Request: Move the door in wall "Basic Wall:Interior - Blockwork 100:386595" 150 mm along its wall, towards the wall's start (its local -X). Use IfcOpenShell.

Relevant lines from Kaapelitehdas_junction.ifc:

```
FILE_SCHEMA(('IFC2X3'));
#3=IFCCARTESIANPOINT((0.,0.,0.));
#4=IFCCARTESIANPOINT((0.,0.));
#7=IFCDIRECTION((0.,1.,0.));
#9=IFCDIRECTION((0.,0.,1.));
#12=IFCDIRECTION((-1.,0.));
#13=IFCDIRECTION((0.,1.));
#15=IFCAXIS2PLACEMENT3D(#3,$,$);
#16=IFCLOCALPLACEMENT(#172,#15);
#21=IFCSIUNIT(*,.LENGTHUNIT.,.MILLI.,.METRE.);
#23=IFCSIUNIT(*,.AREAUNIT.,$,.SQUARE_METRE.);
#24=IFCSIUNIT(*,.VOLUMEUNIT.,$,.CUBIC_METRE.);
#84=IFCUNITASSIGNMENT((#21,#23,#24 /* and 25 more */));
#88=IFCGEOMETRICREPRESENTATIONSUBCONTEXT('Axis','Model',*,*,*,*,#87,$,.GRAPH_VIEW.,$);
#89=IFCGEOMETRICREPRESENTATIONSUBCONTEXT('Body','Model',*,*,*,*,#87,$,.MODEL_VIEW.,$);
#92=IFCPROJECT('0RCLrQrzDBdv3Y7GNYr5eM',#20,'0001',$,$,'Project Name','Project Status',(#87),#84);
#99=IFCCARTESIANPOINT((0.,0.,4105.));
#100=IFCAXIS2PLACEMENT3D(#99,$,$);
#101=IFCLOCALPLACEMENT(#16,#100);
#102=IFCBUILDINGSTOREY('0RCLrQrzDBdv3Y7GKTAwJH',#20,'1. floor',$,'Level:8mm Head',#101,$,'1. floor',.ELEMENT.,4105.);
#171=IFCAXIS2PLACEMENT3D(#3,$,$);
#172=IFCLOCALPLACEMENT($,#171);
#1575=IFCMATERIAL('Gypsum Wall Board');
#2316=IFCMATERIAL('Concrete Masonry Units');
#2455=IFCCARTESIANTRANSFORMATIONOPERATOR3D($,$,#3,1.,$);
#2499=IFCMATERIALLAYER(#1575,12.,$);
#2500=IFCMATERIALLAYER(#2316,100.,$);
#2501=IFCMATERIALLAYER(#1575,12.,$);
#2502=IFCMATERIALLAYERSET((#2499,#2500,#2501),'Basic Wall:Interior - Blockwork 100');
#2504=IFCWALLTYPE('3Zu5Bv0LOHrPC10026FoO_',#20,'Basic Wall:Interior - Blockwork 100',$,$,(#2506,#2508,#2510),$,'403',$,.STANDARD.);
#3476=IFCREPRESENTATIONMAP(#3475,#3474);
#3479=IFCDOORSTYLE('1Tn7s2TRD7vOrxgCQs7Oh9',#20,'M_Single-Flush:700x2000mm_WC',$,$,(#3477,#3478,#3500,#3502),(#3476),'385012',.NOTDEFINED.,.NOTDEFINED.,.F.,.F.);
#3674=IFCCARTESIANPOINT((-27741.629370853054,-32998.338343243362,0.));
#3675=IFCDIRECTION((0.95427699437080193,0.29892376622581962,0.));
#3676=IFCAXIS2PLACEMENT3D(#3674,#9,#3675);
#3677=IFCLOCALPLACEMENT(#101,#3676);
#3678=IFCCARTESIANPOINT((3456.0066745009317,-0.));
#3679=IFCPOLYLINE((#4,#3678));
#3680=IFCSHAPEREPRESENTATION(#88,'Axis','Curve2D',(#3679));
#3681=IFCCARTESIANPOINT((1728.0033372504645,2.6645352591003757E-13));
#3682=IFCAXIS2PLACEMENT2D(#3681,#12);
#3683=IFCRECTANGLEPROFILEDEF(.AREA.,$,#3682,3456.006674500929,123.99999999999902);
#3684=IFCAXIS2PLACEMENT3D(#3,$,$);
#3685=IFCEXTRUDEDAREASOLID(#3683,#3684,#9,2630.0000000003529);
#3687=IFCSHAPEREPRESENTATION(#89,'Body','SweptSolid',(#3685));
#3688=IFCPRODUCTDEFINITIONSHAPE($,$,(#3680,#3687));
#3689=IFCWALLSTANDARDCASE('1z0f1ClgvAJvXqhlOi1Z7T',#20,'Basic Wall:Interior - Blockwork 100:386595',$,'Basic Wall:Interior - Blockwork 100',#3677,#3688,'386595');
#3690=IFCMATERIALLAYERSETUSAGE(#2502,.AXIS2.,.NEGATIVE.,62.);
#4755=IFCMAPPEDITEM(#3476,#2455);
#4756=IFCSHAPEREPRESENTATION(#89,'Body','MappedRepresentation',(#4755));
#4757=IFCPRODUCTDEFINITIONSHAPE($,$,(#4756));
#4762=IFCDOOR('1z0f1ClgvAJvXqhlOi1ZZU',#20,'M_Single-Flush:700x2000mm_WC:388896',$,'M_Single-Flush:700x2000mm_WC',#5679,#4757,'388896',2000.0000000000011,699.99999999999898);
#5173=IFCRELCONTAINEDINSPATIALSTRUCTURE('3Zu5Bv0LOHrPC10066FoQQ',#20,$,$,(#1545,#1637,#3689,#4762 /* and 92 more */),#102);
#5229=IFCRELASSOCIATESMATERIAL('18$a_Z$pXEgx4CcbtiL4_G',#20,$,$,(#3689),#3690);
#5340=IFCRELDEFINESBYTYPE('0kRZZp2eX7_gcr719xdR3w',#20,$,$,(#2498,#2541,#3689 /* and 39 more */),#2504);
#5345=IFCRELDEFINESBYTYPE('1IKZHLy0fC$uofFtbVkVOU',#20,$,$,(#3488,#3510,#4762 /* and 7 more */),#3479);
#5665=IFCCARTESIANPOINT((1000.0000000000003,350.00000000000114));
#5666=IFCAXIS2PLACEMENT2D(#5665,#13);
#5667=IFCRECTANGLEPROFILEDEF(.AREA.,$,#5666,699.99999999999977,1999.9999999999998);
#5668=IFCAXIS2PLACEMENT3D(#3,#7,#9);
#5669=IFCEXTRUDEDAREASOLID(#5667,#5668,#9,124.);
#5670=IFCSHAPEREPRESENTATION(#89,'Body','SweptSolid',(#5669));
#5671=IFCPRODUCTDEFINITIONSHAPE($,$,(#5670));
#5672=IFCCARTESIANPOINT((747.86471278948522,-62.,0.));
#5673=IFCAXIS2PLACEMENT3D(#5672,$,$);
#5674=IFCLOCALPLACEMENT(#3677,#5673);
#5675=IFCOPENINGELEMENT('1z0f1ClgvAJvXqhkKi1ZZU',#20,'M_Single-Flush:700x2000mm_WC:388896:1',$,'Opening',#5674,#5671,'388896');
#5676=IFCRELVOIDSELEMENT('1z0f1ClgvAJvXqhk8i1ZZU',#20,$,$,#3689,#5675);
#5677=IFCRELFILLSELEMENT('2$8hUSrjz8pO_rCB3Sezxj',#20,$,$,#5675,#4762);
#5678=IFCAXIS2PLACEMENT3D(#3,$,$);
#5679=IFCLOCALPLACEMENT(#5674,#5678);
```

```python
import ifcopenshell
import ifcopenshell.api.geometry
import ifcopenshell.util.placement

model = ifcopenshell.open("Kaapelitehdas_junction.ifc")

door = model.by_guid("1z0f1ClgvAJvXqhlOi1ZZU")
opening = door.FillsVoids[0].RelatingOpeningElement
wall = opening.VoidsElements[0].RelatingBuildingElement

wall_matrix = ifcopenshell.util.placement.get_local_placement(wall.ObjectPlacement)
shift = wall_matrix[:3, 0] * -150.0
before = ifcopenshell.util.placement.get_local_placement(door.ObjectPlacement)[:3, 3].copy()

# The door is placed relative to its opening, so it follows when the opening moves.
matrix = ifcopenshell.util.placement.get_local_placement(opening.ObjectPlacement)
matrix[:3, 3] += shift
ifcopenshell.api.geometry.edit_object_placement(
    model, product=opening, matrix=matrix, is_si=False, should_transform_children=True
)

after = ifcopenshell.util.placement.get_local_placement(door.ObjectPlacement)[:3, 3]
print("door moved by", (after - before).round(3) + 0.0)

model.write("Kaapelitehdas_junction_edited.ifc")
```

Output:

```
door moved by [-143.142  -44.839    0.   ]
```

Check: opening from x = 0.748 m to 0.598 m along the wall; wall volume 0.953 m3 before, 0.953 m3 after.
